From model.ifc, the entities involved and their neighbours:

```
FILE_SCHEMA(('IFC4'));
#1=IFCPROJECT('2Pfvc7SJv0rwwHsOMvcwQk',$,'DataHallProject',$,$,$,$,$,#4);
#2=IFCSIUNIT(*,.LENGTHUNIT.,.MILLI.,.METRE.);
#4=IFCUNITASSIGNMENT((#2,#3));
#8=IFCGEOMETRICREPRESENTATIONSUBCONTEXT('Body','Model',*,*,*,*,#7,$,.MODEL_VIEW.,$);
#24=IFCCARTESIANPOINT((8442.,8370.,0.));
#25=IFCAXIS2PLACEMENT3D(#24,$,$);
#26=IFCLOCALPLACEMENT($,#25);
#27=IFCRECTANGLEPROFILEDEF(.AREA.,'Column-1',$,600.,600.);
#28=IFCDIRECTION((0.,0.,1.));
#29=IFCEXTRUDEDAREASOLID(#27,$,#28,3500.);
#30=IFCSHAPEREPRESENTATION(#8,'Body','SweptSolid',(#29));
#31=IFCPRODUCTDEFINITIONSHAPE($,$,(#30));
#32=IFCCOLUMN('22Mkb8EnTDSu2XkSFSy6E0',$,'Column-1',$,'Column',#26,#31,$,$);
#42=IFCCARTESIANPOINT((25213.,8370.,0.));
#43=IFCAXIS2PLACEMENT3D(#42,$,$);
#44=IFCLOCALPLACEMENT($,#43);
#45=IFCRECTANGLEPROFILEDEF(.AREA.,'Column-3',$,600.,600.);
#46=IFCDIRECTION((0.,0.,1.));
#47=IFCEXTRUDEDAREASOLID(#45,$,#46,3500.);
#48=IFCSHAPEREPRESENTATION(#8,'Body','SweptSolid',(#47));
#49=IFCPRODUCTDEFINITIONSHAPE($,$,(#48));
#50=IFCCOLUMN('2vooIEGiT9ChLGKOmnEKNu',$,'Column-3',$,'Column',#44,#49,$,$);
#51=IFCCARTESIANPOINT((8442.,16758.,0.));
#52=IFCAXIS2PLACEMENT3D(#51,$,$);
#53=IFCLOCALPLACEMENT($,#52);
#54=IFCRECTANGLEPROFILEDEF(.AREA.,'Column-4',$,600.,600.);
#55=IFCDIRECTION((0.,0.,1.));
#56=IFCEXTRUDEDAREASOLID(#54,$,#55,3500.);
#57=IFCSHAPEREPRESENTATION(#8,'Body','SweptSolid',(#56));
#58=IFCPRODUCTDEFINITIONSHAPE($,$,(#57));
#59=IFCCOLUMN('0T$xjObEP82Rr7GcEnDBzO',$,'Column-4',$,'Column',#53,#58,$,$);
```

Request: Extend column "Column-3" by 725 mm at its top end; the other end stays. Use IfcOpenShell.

```python
import ifcopenshell
import ifcopenshell.util.representation
import ifcopenshell.util.unit

model = ifcopenshell.open("model.ifc")
unit_scale = ifcopenshell.util.unit.calculate_unit_scale(model)

member = model.by_guid("2vooIEGiT9ChLGKOmnEKNu")
change = 0.725 / unit_scale

# The extrusion runs towards the end named, so only its depth changes.
body = ifcopenshell.util.representation.get_representation(member, "Model", "Body")
solid = body.Items[0]
old_length = solid.Depth
solid.Depth += change

print(f"length {old_length:g} -> {solid.Depth:g}")

model.write("model-out.ifc")
```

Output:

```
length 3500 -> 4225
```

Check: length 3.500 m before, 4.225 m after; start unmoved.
